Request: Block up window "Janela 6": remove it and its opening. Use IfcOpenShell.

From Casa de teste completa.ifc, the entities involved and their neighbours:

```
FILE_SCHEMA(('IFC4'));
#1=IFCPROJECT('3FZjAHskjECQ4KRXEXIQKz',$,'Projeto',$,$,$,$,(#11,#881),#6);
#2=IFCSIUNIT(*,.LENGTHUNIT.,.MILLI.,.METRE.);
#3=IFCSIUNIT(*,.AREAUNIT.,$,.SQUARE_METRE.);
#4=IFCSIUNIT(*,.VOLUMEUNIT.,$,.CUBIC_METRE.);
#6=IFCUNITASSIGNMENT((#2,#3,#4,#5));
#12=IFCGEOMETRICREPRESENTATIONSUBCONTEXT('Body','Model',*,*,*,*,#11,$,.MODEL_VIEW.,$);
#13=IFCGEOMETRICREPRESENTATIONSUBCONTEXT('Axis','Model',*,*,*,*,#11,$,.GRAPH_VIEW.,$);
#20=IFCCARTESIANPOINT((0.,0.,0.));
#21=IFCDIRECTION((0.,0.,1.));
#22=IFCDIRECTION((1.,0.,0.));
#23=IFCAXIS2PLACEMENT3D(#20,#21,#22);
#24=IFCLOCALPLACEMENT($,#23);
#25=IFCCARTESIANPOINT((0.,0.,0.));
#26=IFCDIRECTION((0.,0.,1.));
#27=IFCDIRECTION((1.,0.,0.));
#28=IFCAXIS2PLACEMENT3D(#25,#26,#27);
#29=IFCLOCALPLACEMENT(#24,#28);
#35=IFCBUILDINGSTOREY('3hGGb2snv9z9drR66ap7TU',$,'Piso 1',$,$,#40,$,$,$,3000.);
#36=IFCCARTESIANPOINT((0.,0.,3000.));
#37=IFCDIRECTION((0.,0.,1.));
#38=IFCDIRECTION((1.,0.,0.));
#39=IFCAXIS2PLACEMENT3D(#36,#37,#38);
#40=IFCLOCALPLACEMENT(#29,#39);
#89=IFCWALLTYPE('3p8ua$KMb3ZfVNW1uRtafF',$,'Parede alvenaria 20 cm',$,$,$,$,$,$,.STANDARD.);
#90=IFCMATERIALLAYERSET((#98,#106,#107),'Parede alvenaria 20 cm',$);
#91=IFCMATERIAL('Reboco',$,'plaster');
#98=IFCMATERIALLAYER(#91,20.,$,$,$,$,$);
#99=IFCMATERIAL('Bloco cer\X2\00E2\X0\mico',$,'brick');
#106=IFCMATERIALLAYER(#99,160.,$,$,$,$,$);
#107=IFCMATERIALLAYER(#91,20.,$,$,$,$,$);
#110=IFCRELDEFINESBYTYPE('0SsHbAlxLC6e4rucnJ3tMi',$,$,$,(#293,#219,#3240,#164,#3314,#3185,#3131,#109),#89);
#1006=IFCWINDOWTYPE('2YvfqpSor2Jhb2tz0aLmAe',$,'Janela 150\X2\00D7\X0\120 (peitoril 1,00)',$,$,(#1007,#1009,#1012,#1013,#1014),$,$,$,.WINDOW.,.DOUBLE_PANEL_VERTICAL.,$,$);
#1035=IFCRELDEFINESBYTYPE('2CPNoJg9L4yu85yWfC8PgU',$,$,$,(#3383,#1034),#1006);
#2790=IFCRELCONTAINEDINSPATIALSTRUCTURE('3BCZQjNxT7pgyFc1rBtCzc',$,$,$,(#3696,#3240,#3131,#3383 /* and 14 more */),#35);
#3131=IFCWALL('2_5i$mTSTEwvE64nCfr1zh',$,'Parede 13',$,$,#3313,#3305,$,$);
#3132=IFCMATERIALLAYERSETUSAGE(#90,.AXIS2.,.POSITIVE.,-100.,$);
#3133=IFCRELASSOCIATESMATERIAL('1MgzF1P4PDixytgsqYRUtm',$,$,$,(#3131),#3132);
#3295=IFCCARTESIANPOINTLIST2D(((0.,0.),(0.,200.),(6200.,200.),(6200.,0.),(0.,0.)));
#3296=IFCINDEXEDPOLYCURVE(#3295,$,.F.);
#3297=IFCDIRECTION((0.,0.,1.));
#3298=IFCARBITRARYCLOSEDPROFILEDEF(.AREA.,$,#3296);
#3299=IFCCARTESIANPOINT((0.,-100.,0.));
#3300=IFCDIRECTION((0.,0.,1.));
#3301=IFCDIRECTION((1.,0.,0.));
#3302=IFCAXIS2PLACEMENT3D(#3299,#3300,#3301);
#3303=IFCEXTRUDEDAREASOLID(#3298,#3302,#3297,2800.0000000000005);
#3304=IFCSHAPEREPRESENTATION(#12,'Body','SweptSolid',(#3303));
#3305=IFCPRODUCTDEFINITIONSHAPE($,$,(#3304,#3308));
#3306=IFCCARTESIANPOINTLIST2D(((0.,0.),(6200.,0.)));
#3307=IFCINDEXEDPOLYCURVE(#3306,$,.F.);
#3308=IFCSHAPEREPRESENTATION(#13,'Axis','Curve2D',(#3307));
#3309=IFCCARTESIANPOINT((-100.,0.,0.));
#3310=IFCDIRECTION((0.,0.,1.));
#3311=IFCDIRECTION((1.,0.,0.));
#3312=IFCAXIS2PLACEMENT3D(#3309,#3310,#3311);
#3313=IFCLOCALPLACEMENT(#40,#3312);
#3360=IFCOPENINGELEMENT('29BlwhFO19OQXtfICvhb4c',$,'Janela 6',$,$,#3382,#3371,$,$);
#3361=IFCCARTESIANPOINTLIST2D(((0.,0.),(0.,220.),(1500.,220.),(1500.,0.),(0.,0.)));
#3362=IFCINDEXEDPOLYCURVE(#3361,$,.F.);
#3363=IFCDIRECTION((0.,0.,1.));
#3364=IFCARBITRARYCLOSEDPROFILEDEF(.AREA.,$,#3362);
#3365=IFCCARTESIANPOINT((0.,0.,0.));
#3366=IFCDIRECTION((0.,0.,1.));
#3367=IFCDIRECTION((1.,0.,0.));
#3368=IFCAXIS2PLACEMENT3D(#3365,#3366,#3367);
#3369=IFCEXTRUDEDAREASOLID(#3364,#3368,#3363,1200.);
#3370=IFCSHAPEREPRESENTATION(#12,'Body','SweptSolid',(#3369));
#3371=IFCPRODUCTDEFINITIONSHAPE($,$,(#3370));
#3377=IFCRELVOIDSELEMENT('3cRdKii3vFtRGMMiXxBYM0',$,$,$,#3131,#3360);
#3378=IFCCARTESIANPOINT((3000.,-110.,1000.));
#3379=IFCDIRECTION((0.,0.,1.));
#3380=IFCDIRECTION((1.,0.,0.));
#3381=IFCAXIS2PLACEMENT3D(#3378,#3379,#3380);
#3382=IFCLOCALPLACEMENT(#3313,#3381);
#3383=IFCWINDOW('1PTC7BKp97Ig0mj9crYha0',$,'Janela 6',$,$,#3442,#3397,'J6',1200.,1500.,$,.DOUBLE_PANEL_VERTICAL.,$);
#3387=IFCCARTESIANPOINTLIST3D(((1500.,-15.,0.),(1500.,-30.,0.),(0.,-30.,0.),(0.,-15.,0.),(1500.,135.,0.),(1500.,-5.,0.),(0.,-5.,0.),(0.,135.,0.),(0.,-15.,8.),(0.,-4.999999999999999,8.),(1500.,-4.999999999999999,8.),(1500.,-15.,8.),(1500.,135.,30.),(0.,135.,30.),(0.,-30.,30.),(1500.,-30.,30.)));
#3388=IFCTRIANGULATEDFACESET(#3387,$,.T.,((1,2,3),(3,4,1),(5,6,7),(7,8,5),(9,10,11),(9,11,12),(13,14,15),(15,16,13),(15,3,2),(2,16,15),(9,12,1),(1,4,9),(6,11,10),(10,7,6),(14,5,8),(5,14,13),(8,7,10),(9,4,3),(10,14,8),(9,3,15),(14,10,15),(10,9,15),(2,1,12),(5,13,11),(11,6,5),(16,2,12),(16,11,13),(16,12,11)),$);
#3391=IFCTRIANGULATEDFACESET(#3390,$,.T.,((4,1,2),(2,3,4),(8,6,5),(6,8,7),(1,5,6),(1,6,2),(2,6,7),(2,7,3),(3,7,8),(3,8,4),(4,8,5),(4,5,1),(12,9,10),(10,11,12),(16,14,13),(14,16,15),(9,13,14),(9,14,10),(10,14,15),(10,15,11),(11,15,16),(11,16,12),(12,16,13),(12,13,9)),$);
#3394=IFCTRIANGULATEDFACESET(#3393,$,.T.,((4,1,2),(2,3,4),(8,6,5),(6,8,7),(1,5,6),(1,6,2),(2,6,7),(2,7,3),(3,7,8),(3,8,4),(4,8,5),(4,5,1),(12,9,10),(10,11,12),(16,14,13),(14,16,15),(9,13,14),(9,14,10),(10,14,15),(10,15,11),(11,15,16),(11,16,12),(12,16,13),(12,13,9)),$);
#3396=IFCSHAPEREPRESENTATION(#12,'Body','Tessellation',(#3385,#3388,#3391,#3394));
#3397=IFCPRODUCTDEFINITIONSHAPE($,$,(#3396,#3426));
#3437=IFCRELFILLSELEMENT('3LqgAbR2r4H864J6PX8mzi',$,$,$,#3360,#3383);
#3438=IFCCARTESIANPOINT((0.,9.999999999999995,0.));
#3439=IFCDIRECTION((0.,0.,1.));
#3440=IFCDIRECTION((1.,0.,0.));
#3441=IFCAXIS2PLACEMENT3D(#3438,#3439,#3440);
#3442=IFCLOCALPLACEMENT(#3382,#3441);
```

```python
import ifcopenshell
import ifcopenshell.api.feature
import ifcopenshell.api.root
import ifcopenshell.geom
import ifcopenshell.util.shape

model = ifcopenshell.open("Casa de teste completa.ifc")
settings = ifcopenshell.geom.settings()


def volume(element):
    """Net volume in cubic metres, openings subtracted."""
    shape = ifcopenshell.geom.create_shape(settings, element)
    return ifcopenshell.util.shape.get_volume(shape.geometry)


window = model.by_guid("1PTC7BKp97Ig0mj9crYha0")
opening = window.FillsVoids[0].RelatingOpeningElement
wall = opening.VoidsElements[0].RelatingBuildingElement
before = volume(wall)

ifcopenshell.api.root.remove_product(model, product=window)
ifcopenshell.api.feature.remove_feature(model, feature=opening)

after = volume(wall)

print(f"wall volume {before:.3f} -> {after:.3f} m3")

model.write("Casa de teste completa_updated.ifc")
```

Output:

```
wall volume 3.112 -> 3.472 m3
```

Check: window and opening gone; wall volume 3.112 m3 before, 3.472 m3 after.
